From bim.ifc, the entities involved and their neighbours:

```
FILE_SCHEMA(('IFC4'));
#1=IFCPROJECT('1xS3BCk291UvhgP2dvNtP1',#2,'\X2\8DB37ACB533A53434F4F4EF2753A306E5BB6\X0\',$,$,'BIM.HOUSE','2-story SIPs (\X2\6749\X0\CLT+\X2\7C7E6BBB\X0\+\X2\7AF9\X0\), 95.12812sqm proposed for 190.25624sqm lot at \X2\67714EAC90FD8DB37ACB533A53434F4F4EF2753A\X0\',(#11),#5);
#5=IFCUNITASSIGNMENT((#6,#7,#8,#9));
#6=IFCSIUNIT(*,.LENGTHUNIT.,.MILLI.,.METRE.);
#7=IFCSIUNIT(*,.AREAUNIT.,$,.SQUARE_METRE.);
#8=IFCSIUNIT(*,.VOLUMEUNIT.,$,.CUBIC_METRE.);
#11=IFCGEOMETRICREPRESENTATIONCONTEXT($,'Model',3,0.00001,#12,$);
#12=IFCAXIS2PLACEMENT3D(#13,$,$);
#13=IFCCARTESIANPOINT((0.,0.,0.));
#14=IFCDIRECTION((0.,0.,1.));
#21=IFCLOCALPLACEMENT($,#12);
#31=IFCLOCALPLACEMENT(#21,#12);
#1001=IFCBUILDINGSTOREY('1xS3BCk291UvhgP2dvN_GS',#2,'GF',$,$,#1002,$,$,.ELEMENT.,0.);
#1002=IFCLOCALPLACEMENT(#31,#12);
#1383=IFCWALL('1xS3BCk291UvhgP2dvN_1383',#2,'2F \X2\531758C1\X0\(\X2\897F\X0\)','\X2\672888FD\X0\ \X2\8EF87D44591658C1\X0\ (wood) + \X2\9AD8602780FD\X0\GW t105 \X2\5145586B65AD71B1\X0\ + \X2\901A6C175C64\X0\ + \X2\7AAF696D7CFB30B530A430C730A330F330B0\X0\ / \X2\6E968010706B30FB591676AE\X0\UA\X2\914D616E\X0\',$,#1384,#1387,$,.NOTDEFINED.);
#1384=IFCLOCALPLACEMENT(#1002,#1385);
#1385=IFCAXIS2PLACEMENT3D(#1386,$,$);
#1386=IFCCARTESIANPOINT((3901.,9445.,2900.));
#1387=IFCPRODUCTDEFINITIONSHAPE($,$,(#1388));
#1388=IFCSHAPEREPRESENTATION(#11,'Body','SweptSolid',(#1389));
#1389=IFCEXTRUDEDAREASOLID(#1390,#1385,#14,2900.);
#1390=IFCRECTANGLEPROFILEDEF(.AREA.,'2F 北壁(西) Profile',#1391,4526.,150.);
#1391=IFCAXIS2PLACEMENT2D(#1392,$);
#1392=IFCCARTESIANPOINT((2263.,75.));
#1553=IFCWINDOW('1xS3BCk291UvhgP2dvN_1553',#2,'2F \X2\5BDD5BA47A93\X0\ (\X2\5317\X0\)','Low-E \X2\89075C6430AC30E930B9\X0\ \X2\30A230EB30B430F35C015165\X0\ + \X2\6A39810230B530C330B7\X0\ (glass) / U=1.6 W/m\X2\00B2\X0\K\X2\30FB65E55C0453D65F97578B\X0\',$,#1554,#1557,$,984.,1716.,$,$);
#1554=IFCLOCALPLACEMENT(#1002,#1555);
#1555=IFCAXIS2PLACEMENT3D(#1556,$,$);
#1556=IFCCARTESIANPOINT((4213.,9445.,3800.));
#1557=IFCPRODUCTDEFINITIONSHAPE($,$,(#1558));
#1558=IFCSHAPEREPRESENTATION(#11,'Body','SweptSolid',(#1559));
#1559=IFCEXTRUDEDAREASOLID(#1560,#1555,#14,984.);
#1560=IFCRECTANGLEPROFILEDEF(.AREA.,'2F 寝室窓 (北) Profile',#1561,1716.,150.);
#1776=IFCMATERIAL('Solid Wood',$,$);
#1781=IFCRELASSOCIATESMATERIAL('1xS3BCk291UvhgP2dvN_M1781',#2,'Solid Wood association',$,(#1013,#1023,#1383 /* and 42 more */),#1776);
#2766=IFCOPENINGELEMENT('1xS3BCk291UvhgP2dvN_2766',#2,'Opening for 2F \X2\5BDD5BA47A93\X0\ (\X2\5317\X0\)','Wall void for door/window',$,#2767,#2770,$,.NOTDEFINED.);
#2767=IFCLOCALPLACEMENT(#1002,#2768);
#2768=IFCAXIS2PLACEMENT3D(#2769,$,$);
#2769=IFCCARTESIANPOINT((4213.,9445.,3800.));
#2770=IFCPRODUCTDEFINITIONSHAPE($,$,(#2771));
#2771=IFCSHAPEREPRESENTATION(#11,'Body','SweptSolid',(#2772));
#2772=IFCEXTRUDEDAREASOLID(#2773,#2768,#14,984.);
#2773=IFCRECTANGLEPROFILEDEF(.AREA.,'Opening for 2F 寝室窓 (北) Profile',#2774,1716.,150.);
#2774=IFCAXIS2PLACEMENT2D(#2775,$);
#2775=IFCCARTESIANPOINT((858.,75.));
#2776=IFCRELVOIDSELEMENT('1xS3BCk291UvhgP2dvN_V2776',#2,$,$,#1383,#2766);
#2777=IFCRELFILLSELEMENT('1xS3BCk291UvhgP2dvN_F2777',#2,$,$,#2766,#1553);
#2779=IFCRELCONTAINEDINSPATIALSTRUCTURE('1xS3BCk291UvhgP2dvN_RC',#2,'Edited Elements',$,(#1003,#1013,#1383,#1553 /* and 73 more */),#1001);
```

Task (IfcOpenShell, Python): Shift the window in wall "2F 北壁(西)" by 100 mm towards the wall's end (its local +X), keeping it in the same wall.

```python
import ifcopenshell
import ifcopenshell.api.geometry
import ifcopenshell.util.placement

model = ifcopenshell.open("bim.ifc")

window = model.by_guid("1xS3BCk291UvhgP2dvN_1553")
opening = window.FillsVoids[0].RelatingOpeningElement
wall = opening.VoidsElements[0].RelatingBuildingElement

wall_matrix = ifcopenshell.util.placement.get_local_placement(wall.ObjectPlacement)
shift = wall_matrix[:3, 0] * 100.0
before = ifcopenshell.util.placement.get_local_placement(window.ObjectPlacement)[:3, 3].copy()

# The window is not placed relative to its opening, so move both.
for product in (opening, window):
    matrix = ifcopenshell.util.placement.get_local_placement(product.ObjectPlacement)
    matrix[:3, 3] += shift
    ifcopenshell.api.geometry.edit_object_placement(model, product=product, matrix=matrix, is_si=False)

after = ifcopenshell.util.placement.get_local_placement(window.ObjectPlacement)[:3, 3]
print("window moved by", (after - before).round(3) + 0.0)

model.write("bim_v2.ifc")
```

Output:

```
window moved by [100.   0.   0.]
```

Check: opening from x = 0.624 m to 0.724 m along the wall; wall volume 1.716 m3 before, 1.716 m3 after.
